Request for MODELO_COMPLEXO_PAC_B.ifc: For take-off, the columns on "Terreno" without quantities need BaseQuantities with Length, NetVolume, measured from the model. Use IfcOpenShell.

First a look at what the model holds.

```python
import ifcopenshell
import ifcopenshell.util.element
import ifcopenshell.util.unit

model = ifcopenshell.open("MODELO_COMPLEXO_PAC_B.ifc")
print(model.schema)
for unit_type in ("LENGTHUNIT", "AREAUNIT", "VOLUMEUNIT"):
    print(unit_type, ifcopenshell.util.unit.calculate_unit_scale(model, unit_type))
storey = next(s for s in model.by_type("IfcBuildingStorey") if s.Name == "Terreno")
columns = [e for e in ifcopenshell.util.element.get_decomposition(storey) if e.is_a("IfcColumn")]
for e in sorted(columns, key=lambda e: e.id()):
    print(e.id(), e.is_a(), e.Name, list(ifcopenshell.util.element.get_psets(e, qtos_only=True)), sep=" | ")
```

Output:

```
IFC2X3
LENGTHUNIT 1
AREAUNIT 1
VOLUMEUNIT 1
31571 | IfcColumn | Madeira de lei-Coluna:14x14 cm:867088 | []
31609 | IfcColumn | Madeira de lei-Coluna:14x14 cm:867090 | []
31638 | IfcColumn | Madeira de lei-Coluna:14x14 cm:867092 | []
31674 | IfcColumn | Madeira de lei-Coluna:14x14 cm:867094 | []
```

```python
import ifcopenshell
import ifcopenshell.api.pset
import ifcopenshell.geom
import ifcopenshell.util.element
import ifcopenshell.util.shape
import ifcopenshell.util.unit

model = ifcopenshell.open("MODELO_COMPLEXO_PAC_B.ifc")
unit_scale = ifcopenshell.util.unit.calculate_unit_scale(model)
volume_scale = ifcopenshell.util.unit.calculate_unit_scale(model, "VOLUMEUNIT")
settings = ifcopenshell.geom.settings()

storey = next(s for s in model.by_type("IfcBuildingStorey") if s.Name == "Terreno")
columns = [e for e in ifcopenshell.util.element.get_decomposition(storey) if e.is_a("IfcColumn")]

for e in sorted(columns, key=lambda e: e.id()):
    if ifcopenshell.util.element.get_psets(e, qtos_only=True, should_inherit=False):
        continue
    # Geometry comes back in metres, in the element's own axes.
    shape = ifcopenshell.geom.create_shape(settings, e)
    values = {
        "Length": ifcopenshell.util.shape.get_z(shape.geometry) / unit_scale,
        "NetVolume": ifcopenshell.util.shape.get_volume(shape.geometry) / volume_scale,
    }
    qto = ifcopenshell.api.pset.add_qto(model, product=e, name="BaseQuantities")
    ifcopenshell.api.pset.edit_qto(model, qto=qto, properties=values)
    print(e.id(), {k: round(v, 3) for k, v in values.items()})

model.write("MODELO_COMPLEXO_PAC_B_v2.ifc")
```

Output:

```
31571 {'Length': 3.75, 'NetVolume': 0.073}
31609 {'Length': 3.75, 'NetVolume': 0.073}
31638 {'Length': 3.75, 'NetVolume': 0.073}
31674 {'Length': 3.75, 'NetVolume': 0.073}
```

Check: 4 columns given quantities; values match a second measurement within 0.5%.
